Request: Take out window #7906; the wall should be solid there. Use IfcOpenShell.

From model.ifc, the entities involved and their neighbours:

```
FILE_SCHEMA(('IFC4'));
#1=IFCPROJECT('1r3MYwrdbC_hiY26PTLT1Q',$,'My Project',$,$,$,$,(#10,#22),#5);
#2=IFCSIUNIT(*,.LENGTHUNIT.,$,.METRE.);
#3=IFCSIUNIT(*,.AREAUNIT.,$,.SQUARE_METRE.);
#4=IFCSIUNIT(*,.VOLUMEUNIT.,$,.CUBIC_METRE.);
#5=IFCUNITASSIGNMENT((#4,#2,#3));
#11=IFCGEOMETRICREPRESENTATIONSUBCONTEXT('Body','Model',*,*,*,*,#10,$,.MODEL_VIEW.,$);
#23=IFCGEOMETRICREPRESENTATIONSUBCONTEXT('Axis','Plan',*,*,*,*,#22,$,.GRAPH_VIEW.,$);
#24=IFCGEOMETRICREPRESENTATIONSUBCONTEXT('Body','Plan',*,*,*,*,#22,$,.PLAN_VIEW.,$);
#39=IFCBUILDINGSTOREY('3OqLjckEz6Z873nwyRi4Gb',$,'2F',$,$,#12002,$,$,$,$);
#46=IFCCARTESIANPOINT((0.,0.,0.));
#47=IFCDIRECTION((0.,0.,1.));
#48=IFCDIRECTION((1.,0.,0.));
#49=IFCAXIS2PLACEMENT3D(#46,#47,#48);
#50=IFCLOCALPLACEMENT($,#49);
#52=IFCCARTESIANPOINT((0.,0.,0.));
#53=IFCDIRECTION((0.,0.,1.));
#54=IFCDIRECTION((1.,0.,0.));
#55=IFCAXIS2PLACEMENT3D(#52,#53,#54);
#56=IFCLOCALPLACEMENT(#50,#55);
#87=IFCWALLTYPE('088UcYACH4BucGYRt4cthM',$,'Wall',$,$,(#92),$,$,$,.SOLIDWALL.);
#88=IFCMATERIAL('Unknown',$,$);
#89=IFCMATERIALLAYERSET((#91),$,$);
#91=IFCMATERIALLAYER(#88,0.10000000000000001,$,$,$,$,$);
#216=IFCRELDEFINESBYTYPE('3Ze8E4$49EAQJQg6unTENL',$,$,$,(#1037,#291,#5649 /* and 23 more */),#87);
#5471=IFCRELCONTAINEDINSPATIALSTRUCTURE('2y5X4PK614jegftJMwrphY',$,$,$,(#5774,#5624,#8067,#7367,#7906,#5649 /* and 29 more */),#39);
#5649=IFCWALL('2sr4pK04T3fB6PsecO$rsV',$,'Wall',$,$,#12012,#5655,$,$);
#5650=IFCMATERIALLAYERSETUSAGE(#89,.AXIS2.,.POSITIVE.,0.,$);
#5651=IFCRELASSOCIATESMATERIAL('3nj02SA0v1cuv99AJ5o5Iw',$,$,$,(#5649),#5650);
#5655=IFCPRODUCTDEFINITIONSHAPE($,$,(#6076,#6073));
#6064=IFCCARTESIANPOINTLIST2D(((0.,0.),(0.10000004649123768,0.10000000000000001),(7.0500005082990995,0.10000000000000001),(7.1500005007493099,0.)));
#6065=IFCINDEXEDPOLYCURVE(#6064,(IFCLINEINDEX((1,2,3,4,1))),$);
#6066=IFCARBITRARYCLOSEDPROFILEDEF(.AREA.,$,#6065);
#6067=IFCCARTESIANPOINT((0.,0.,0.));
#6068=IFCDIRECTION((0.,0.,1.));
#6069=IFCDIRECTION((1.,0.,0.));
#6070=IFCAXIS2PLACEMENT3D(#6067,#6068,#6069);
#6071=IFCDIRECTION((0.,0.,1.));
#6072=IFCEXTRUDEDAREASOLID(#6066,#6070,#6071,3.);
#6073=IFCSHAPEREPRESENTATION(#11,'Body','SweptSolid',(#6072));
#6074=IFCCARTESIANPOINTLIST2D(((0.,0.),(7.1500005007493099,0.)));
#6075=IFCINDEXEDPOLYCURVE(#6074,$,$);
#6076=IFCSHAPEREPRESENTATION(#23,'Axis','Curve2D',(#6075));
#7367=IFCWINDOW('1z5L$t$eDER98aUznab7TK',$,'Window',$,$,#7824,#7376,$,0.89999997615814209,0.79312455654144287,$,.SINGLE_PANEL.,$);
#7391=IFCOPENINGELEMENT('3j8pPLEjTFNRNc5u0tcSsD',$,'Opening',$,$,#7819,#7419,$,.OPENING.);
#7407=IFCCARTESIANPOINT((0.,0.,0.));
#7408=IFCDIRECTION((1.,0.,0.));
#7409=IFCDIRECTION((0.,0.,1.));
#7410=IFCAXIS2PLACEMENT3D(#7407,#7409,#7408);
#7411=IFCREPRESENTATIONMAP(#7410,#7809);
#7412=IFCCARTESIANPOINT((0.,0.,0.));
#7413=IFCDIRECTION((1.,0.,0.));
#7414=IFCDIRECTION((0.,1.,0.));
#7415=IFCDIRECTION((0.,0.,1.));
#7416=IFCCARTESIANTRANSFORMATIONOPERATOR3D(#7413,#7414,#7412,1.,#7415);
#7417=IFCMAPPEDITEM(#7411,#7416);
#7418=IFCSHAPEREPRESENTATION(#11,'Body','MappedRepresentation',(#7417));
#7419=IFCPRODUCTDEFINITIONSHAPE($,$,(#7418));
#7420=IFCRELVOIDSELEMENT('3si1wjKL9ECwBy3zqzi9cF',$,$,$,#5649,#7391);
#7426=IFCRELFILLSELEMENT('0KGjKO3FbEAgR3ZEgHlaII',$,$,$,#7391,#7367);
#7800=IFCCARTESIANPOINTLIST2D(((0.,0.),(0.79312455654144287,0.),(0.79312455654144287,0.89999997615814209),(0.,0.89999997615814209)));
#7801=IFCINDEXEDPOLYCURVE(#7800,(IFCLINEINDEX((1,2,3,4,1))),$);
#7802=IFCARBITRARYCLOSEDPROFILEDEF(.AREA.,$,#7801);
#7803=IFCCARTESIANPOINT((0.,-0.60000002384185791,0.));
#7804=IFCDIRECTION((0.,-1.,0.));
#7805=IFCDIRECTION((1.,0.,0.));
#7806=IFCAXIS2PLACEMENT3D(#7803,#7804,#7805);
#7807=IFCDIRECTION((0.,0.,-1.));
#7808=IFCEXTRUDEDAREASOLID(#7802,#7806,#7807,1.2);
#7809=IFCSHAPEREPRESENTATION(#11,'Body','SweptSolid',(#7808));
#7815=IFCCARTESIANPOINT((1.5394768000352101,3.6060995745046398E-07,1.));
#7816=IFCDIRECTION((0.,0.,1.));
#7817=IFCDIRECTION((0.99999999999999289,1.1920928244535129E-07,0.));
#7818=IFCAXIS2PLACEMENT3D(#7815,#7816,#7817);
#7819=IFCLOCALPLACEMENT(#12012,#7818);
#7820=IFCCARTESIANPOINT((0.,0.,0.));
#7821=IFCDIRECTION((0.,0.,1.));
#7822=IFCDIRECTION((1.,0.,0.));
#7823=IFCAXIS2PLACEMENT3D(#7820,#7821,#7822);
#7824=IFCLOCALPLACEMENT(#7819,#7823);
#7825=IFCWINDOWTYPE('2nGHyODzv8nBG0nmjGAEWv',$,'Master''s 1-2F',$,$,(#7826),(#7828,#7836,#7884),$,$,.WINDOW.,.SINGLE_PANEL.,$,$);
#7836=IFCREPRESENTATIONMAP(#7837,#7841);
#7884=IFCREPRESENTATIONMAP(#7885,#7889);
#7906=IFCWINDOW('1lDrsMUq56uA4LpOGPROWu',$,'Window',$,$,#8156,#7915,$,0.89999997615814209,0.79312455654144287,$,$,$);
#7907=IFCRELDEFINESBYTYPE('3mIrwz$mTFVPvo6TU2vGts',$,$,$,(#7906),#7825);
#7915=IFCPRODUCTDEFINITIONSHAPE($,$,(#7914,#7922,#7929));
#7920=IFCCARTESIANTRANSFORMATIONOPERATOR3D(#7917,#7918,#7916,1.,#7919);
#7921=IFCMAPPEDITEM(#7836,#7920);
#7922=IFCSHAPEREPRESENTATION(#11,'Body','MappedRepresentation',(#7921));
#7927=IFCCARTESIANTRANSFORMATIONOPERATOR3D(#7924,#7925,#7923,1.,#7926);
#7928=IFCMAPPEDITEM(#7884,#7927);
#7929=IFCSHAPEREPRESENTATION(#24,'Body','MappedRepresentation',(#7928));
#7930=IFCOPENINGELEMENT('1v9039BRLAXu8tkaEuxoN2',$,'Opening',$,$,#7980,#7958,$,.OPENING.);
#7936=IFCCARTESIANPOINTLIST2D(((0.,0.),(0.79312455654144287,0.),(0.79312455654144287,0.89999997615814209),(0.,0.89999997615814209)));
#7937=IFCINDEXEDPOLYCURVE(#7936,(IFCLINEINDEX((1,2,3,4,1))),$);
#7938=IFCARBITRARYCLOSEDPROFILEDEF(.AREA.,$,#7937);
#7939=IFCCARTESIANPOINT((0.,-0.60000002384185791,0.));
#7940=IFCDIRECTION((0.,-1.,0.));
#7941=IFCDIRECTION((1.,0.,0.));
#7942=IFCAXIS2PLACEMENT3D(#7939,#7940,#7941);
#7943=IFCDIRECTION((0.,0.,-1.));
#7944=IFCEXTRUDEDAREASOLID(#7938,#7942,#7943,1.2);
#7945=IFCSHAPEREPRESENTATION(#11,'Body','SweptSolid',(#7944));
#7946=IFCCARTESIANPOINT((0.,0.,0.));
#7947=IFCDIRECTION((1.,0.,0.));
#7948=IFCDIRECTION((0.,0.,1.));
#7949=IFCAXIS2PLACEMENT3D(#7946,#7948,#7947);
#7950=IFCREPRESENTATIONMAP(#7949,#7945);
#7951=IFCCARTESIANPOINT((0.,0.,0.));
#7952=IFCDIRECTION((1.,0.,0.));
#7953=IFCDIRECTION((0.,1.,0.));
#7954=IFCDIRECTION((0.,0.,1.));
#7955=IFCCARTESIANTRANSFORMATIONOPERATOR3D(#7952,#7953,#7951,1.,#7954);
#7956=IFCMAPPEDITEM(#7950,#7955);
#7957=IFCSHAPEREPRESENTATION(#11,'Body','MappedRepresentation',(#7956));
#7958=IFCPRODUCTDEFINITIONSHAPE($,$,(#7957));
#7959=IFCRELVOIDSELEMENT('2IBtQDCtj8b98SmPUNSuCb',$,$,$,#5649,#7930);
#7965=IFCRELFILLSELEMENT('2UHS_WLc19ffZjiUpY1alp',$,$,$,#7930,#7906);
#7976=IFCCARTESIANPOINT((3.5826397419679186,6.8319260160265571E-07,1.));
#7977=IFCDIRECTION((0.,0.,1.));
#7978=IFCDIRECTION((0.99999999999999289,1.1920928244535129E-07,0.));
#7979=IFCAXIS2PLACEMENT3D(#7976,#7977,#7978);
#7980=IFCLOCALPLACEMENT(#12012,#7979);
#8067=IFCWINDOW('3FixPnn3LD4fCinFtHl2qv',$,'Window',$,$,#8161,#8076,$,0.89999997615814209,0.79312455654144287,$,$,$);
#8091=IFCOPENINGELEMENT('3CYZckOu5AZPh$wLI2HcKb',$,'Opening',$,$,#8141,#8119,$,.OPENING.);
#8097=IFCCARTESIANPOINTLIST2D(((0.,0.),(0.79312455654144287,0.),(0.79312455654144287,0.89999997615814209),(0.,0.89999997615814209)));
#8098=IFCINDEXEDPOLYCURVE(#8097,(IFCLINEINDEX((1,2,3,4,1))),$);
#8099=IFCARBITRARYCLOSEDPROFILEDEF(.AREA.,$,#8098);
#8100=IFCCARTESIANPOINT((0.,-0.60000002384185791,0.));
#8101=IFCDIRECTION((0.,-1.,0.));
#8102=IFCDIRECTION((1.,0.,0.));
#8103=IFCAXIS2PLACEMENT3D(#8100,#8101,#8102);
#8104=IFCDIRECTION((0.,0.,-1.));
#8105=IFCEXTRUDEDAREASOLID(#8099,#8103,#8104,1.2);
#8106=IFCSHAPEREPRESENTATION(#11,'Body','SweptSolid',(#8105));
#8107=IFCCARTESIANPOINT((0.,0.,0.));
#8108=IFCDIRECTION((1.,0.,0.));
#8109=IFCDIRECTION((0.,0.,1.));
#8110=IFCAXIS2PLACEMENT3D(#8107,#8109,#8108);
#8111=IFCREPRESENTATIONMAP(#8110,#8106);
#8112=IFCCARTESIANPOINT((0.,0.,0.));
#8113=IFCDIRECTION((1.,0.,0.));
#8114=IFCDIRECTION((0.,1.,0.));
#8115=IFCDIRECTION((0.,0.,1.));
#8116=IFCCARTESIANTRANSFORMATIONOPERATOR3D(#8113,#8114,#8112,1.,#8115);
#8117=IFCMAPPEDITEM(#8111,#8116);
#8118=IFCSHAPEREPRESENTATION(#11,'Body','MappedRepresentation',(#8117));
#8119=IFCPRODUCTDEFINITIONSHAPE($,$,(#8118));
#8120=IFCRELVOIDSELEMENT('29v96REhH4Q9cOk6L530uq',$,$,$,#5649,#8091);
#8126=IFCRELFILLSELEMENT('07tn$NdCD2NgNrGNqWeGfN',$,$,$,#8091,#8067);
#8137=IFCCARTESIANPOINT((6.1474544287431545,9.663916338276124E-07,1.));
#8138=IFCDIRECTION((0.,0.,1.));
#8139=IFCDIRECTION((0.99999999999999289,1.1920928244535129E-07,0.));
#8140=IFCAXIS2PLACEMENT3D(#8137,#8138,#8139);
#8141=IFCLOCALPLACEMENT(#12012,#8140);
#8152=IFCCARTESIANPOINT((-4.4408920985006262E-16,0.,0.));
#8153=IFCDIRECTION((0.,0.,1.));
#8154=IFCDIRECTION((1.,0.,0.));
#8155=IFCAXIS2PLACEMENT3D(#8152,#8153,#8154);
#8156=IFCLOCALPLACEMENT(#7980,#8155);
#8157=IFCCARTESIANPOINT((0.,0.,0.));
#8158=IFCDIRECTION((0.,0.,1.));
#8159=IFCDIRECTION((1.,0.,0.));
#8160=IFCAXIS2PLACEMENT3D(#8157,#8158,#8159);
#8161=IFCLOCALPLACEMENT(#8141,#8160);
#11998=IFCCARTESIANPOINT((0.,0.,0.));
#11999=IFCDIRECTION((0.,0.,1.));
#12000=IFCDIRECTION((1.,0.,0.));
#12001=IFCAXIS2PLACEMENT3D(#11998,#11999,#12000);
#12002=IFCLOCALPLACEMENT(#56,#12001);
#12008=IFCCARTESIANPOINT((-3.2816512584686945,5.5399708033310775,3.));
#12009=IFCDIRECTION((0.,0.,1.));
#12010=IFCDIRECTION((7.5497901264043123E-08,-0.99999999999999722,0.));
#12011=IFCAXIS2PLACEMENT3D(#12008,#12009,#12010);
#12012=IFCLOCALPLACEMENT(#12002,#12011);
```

```python
import ifcopenshell
import ifcopenshell.api.feature
import ifcopenshell.api.root
import ifcopenshell.geom
import ifcopenshell.util.shape

model = ifcopenshell.open("model.ifc")
settings = ifcopenshell.geom.settings()


def volume(element):
    """Net volume in cubic metres, openings subtracted."""
    shape = ifcopenshell.geom.create_shape(settings, element)
    return ifcopenshell.util.shape.get_volume(shape.geometry)


window = model.by_guid("1lDrsMUq56uA4LpOGPROWu")
opening = window.FillsVoids[0].RelatingOpeningElement
wall = opening.VoidsElements[0].RelatingBuildingElement
before = volume(wall)

ifcopenshell.api.root.remove_product(model, product=window)
ifcopenshell.api.feature.remove_feature(model, feature=opening)

after = volume(wall)

print(f"wall volume {before:.3f} -> {after:.3f} m3")

model.write("model_edited.ifc")
```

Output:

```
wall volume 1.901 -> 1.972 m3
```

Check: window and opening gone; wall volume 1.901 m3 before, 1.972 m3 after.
